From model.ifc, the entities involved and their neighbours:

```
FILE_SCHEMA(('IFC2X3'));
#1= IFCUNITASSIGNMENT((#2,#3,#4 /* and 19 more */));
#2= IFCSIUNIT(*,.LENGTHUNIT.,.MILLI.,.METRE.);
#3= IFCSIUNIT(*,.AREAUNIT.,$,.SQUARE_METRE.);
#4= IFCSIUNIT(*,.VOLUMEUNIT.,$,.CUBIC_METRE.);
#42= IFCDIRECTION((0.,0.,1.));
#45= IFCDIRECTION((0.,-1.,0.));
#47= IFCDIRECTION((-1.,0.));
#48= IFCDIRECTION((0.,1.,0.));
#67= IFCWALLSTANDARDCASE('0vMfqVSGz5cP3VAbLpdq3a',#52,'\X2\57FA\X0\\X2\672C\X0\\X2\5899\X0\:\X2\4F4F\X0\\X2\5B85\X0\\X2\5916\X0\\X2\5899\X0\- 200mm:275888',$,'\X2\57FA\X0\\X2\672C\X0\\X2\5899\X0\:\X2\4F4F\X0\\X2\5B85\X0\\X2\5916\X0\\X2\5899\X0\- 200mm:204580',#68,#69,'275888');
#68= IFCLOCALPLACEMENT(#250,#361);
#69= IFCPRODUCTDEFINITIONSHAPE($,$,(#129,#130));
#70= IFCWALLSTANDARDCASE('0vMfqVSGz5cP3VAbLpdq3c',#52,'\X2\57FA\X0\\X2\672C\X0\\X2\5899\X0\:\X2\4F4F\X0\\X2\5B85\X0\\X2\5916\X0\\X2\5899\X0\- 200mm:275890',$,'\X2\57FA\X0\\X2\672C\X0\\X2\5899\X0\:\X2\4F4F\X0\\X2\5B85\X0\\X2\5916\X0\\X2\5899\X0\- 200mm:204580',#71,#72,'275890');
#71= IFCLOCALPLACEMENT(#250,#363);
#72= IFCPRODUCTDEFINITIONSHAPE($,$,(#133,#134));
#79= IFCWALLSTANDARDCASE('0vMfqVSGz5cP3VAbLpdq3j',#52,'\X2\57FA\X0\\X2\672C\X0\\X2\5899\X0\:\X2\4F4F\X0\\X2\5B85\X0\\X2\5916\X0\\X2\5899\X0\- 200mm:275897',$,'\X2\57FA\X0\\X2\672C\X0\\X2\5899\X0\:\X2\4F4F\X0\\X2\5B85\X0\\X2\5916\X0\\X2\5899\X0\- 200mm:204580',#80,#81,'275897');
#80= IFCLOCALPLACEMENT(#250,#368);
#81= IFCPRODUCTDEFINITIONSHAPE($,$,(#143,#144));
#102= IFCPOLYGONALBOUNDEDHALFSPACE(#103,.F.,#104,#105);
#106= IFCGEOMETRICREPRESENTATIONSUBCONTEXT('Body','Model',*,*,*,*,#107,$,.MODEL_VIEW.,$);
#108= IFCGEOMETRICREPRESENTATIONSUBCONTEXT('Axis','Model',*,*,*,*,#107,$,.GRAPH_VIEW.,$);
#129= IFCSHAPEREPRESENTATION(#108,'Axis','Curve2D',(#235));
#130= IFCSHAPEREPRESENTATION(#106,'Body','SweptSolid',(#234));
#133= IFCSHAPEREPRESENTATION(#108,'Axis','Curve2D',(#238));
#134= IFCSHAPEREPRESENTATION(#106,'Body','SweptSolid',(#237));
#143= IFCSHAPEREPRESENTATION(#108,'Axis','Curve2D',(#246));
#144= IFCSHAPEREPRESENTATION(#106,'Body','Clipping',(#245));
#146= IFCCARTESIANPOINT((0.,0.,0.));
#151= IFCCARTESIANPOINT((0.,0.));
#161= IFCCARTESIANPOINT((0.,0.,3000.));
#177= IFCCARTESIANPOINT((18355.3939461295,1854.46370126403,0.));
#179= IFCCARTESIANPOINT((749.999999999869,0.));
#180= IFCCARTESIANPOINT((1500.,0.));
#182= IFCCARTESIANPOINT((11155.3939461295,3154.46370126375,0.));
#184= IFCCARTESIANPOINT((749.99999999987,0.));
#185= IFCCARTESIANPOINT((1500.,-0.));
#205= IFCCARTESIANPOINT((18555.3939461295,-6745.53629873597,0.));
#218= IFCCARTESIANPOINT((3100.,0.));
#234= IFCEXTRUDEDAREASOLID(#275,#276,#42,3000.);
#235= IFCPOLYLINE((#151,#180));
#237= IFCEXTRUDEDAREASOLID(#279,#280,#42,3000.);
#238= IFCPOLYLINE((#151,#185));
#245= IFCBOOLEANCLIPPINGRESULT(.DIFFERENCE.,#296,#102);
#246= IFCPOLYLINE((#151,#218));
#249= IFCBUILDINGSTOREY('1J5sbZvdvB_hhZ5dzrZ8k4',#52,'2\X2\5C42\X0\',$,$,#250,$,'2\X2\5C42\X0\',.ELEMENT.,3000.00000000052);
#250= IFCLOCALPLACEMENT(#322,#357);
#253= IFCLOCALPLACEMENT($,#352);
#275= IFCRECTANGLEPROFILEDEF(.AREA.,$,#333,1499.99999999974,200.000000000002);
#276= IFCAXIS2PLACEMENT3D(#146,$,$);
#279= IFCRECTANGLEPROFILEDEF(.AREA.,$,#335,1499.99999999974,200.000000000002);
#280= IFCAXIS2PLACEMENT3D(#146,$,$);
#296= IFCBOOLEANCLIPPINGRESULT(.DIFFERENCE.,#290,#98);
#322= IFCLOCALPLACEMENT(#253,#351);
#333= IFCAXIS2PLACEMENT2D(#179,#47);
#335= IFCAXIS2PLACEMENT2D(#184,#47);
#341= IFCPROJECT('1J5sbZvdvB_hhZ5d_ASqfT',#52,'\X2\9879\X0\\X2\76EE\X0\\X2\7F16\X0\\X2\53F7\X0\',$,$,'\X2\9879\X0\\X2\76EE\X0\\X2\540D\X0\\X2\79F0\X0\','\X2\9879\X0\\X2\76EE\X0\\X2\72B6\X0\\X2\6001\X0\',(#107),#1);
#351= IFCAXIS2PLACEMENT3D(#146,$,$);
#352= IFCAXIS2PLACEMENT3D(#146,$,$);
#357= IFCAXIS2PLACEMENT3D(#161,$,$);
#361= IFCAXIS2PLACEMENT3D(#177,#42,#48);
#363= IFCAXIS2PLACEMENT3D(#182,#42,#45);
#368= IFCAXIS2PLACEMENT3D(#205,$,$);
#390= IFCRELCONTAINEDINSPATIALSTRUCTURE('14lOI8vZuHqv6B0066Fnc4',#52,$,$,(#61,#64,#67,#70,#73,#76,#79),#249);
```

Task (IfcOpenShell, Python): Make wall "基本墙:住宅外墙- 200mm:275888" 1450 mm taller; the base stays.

```python
import ifcopenshell
import ifcopenshell.geom
import ifcopenshell.util.representation
import ifcopenshell.util.shape
import ifcopenshell.util.unit

model = ifcopenshell.open("model.ifc")
unit_scale = ifcopenshell.util.unit.calculate_unit_scale(model)
settings = ifcopenshell.geom.settings()


def volume(element):
    """Net volume in cubic metres, openings subtracted."""
    shape = ifcopenshell.geom.create_shape(settings, element)
    return ifcopenshell.util.shape.get_volume(shape.geometry)


wall = model.by_guid("0vMfqVSGz5cP3VAbLpdq3a")
before = volume(wall)

body = ifcopenshell.util.representation.get_representation(wall, "Model", "Body")
solid = body.Items[0]
old_height = solid.Depth
solid.Depth += 1.45 / unit_scale
after = volume(wall)

print(f"height {old_height:g} -> {solid.Depth:g}, volume {before:.3f} -> {after:.3f} m3")

model.write("model-out.ifc")
```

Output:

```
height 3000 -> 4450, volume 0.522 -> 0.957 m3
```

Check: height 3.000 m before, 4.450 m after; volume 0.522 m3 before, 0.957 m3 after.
